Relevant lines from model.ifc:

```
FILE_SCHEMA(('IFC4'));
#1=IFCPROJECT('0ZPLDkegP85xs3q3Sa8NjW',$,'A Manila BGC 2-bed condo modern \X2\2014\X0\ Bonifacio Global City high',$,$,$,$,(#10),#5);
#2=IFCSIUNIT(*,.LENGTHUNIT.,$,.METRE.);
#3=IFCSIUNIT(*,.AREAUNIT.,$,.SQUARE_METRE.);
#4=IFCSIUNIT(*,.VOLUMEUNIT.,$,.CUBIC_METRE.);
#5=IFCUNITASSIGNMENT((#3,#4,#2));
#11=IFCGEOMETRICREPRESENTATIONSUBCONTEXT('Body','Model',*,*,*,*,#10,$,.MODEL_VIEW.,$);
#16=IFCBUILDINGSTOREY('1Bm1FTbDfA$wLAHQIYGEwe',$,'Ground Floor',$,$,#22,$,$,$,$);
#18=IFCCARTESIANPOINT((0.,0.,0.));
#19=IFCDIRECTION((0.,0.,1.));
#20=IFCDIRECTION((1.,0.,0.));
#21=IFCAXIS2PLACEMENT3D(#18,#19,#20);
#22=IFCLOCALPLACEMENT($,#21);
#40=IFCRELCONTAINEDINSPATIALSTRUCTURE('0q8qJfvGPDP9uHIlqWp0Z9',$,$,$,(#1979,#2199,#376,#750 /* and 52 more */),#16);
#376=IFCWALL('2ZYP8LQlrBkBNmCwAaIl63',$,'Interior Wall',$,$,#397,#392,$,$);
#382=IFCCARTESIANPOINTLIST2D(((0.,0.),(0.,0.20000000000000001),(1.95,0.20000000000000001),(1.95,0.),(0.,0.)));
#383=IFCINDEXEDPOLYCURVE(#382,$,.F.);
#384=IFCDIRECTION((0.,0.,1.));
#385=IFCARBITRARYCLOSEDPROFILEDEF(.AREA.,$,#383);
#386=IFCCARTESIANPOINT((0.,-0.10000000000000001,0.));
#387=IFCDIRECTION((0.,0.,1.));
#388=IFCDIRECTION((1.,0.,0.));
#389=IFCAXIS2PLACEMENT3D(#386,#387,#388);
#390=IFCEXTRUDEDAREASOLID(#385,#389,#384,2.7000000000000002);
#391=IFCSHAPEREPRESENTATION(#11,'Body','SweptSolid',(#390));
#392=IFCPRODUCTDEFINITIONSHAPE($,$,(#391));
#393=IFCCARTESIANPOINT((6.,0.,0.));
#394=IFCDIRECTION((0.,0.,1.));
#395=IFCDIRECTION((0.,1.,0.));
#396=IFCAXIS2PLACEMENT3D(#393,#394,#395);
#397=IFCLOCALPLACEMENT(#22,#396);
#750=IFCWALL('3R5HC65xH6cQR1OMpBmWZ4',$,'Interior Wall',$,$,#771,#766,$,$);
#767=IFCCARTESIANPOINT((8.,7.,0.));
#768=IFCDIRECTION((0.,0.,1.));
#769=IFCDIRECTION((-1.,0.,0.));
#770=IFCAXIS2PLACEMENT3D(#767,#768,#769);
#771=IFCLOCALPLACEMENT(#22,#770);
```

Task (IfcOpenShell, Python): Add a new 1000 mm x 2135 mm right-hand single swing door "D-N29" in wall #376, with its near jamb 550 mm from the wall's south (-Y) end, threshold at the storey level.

```python
import numpy as np
import ifcopenshell
import ifcopenshell.api.feature
import ifcopenshell.api.geometry
import ifcopenshell.api.root
import ifcopenshell.api.spatial
import ifcopenshell.geom
import ifcopenshell.util.element
import ifcopenshell.util.placement
import ifcopenshell.util.representation
import ifcopenshell.util.shape
import ifcopenshell.util.unit

model = ifcopenshell.open("model.ifc")
unit_scale = ifcopenshell.util.unit.calculate_unit_scale(model)
settings = ifcopenshell.geom.settings()


def volume(element):
    """Net volume in cubic metres, openings subtracted."""
    shape = ifcopenshell.geom.create_shape(settings, element)
    return ifcopenshell.util.shape.get_volume(shape.geometry)


wall = model.by_id(376)
storey = ifcopenshell.util.element.get_container(wall, ifc_class="IfcBuildingStorey")
context = ifcopenshell.util.representation.get_context(model, "Model", "Body", "MODEL_VIEW")
before = volume(wall)

width, height, from_end, sill = 1, 2.135, 0.55, 0.0  # metres

# The wall runs along its own X axis, and the end named is its -X end.
wall_shape = ifcopenshell.geom.create_shape(settings, wall)
x, y, z = ifcopenshell.util.shape.get_vertices(wall_shape.geometry).T
start = x.min() + from_end
face, thickness = float(y.min()), float(y.max() - y.min())
wall_matrix = ifcopenshell.util.placement.get_local_placement(wall.ObjectPlacement)
level = ifcopenshell.util.placement.get_local_placement(storey.ObjectPlacement)[2, 3]


def in_wall(x, y):
    """Placement at x, y metres in the wall's axes, at sill height."""
    matrix = wall_matrix.copy()
    matrix[:, 3] = wall_matrix @ np.array([x / unit_scale, y / unit_scale, 0.0, 1.0])
    matrix[2, 3] = level + sill / unit_scale
    return matrix


# Opening: a box that overshoots both wall faces by 50 mm.
opening = ifcopenshell.api.root.create_entity(model, ifc_class="IfcOpeningElement", predefined_type="OPENING")
box = ifcopenshell.api.geometry.add_wall_representation(
    model, context=context, length=width, height=height, thickness=thickness + 0.1
)
ifcopenshell.api.geometry.assign_representation(model, product=opening, representation=box)
ifcopenshell.api.geometry.edit_object_placement(model, product=opening, matrix=in_wall(start, face - 0.05), is_si=False)
ifcopenshell.api.feature.add_feature(model, feature=opening, element=wall)

door = ifcopenshell.api.root.create_entity(model, ifc_class="IfcDoor", name="D-N29", predefined_type="DOOR")
door.OverallWidth, door.OverallHeight = width / unit_scale, height / unit_scale
door.OperationType = "SINGLE_SWING_RIGHT"
body = ifcopenshell.api.geometry.add_door_representation(
    model,
    context=context,
    overall_width=door.OverallWidth,
    overall_height=door.OverallHeight,
    operation_type="SINGLE_SWING_RIGHT",
    lining_properties={"LiningDepth": thickness / unit_scale, "ThresholdDepth": thickness / unit_scale},
)
ifcopenshell.api.geometry.assign_representation(model, product=door, representation=body)
ifcopenshell.api.spatial.assign_container(model, products=[door], relating_structure=storey)
ifcopenshell.api.feature.add_filling(model, opening=opening, element=door)

# The lining spans the wall, so the door starts at the wall face.
ifcopenshell.api.geometry.edit_object_placement(model, product=door, matrix=in_wall(start, face), is_si=False)

after = volume(wall)

print(f"wall volume {before:.3f} -> {after:.3f} m3")

model.write("model_rev.ifc")
```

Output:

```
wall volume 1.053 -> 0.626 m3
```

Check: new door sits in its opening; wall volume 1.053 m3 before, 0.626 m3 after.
